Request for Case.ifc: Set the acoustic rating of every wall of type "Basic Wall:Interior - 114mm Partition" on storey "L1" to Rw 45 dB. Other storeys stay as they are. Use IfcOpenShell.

First a look at what the model holds.

```python
import ifcopenshell
import ifcopenshell.util.element

model = ifcopenshell.open("Case.ifc")
print(model.schema)
storey = next(s for s in model.by_type("IfcBuildingStorey") if s.Name == "L1")
walls = [e for e in ifcopenshell.util.element.get_decomposition(storey) if e.is_a("IfcWall")]
seen = {}
for e in walls:
    element_type = ifcopenshell.util.element.get_type(e)
    key = (element_type.Name if element_type != e and element_type else None, ifcopenshell.util.element.get_pset(e, "Pset_WallCommon", "AcousticRating"))
    seen[key] = seen.get(key, 0) + 1
for (name, value), count in sorted(seen.items(), key=str):
    print(count, "x", name, "|", value)
```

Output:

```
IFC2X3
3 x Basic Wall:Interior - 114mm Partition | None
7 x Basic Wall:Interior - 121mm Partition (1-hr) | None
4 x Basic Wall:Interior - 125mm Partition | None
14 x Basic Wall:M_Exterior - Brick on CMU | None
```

```python
import ifcopenshell
import ifcopenshell.api.pset
import ifcopenshell.util.element

model = ifcopenshell.open("Case.ifc")

storey = next(s for s in model.by_type("IfcBuildingStorey") if s.Name == "L1")
walls = [e for e in ifcopenshell.util.element.get_decomposition(storey) if e.is_a("IfcWall")]

count = 0
for e in walls:
    element_type = ifcopenshell.util.element.get_type(e)
    if element_type in (None, e) or element_type.Name != "Basic Wall:Interior - 114mm Partition":
        continue
    # add_pset returns the element's existing set when there is one.
    pset = ifcopenshell.api.pset.add_pset(model, product=e, name="Pset_WallCommon")
    ifcopenshell.api.pset.edit_pset(model, pset=pset, properties={"AcousticRating": "Rw 45 dB"})
    count += 1

print(count, "walls updated")

model.write("Case_rev.ifc")
```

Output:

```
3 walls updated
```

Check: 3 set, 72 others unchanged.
